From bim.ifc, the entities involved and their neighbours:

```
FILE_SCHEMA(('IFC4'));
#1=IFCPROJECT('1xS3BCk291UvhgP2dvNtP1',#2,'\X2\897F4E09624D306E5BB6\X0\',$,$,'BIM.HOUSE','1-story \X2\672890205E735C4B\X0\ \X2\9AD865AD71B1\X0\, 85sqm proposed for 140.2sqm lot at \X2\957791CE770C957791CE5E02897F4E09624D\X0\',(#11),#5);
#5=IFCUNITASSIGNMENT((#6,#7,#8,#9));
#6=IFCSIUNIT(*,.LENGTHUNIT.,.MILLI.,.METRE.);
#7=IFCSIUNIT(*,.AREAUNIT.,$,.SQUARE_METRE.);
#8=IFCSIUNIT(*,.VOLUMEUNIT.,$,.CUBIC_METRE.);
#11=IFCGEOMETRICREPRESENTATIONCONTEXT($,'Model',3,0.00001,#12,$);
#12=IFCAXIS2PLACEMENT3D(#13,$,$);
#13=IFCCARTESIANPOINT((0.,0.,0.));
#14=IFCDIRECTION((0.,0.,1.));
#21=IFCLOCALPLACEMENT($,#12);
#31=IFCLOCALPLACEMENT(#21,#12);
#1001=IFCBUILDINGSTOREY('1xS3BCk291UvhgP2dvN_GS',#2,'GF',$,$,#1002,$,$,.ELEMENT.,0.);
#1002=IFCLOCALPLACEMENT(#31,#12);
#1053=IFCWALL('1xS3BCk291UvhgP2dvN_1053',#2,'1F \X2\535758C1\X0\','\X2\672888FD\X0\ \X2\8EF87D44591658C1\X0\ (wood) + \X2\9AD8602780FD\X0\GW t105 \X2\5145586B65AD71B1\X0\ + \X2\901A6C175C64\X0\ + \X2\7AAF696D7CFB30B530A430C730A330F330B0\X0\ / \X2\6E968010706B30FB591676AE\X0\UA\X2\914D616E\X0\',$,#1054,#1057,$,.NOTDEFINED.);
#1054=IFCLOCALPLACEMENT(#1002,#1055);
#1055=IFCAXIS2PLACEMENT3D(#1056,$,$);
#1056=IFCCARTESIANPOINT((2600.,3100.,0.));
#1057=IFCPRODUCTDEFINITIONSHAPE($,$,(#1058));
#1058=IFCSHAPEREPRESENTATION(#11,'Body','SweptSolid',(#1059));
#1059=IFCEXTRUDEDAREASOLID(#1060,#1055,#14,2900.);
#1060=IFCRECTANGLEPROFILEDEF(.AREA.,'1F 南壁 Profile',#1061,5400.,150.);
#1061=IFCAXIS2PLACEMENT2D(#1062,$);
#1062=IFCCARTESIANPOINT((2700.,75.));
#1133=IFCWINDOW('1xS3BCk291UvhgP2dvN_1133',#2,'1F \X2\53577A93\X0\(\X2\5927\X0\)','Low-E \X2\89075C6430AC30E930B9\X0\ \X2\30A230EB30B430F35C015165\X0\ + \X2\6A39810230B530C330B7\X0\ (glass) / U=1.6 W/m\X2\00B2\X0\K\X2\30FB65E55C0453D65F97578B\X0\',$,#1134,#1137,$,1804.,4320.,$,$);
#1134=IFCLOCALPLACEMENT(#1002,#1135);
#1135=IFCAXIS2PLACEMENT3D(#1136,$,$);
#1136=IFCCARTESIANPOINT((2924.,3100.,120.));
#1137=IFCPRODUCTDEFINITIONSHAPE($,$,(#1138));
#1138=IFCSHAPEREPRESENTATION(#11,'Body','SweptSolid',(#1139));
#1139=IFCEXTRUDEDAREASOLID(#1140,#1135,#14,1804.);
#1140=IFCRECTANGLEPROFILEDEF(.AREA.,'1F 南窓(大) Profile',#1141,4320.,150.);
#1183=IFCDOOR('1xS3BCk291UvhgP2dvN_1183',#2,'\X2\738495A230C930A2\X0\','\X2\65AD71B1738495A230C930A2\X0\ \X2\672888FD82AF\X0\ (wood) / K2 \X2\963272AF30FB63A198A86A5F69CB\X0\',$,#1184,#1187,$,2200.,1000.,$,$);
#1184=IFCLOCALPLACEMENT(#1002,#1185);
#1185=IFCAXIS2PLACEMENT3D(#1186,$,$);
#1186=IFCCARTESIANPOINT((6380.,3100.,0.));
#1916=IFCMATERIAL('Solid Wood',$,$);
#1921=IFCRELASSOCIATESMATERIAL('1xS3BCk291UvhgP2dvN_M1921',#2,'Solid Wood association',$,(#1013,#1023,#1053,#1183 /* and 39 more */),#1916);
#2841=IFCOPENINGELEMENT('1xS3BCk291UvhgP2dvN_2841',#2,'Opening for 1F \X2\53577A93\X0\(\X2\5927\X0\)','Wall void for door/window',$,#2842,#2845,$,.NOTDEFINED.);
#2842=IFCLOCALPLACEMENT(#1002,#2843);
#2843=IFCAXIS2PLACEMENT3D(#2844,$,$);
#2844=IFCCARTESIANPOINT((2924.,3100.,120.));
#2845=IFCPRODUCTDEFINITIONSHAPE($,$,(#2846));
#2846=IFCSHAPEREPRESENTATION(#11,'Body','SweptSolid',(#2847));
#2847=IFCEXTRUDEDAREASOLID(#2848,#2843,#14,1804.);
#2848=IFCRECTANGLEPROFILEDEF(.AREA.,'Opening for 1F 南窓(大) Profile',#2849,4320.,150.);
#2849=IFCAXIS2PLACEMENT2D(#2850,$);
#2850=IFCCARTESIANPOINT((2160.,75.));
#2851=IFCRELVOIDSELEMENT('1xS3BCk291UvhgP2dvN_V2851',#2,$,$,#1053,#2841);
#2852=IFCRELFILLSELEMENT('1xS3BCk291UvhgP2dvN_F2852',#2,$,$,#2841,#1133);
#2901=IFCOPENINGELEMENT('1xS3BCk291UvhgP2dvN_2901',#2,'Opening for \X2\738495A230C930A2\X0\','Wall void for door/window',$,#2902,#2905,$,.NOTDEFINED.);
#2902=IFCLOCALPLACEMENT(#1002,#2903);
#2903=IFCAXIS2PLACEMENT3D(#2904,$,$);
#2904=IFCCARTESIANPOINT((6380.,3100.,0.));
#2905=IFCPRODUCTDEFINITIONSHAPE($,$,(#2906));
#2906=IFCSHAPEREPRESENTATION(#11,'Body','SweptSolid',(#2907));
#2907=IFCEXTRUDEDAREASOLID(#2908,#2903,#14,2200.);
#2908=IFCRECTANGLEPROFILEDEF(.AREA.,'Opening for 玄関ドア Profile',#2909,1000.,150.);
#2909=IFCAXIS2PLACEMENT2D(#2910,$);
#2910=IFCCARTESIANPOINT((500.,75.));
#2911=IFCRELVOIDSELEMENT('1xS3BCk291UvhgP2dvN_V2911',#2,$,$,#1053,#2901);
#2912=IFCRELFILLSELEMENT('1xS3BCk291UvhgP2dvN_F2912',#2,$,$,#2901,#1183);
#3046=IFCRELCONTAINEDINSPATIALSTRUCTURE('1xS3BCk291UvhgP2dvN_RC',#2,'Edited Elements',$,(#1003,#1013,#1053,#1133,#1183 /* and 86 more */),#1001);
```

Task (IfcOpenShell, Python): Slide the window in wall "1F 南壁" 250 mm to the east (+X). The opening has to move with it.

```python
import ifcopenshell
import ifcopenshell.api.geometry
import ifcopenshell.util.placement

model = ifcopenshell.open("bim.ifc")

window = model.by_guid("1xS3BCk291UvhgP2dvN_1133")
opening = window.FillsVoids[0].RelatingOpeningElement
wall = opening.VoidsElements[0].RelatingBuildingElement

wall_matrix = ifcopenshell.util.placement.get_local_placement(wall.ObjectPlacement)
shift = wall_matrix[:3, 0] * 250.0
before = ifcopenshell.util.placement.get_local_placement(window.ObjectPlacement)[:3, 3].copy()

# The window is not placed relative to its opening, so move both.
for product in (opening, window):
    matrix = ifcopenshell.util.placement.get_local_placement(product.ObjectPlacement)
    matrix[:3, 3] += shift
    ifcopenshell.api.geometry.edit_object_placement(model, product=product, matrix=matrix, is_si=False)

after = ifcopenshell.util.placement.get_local_placement(window.ObjectPlacement)[:3, 3]
print("window moved by", (after - before).round(3) + 0.0)

model.write("bim-out.ifc")
```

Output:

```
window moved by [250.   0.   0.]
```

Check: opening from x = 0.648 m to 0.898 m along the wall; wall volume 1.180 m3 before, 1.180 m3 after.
